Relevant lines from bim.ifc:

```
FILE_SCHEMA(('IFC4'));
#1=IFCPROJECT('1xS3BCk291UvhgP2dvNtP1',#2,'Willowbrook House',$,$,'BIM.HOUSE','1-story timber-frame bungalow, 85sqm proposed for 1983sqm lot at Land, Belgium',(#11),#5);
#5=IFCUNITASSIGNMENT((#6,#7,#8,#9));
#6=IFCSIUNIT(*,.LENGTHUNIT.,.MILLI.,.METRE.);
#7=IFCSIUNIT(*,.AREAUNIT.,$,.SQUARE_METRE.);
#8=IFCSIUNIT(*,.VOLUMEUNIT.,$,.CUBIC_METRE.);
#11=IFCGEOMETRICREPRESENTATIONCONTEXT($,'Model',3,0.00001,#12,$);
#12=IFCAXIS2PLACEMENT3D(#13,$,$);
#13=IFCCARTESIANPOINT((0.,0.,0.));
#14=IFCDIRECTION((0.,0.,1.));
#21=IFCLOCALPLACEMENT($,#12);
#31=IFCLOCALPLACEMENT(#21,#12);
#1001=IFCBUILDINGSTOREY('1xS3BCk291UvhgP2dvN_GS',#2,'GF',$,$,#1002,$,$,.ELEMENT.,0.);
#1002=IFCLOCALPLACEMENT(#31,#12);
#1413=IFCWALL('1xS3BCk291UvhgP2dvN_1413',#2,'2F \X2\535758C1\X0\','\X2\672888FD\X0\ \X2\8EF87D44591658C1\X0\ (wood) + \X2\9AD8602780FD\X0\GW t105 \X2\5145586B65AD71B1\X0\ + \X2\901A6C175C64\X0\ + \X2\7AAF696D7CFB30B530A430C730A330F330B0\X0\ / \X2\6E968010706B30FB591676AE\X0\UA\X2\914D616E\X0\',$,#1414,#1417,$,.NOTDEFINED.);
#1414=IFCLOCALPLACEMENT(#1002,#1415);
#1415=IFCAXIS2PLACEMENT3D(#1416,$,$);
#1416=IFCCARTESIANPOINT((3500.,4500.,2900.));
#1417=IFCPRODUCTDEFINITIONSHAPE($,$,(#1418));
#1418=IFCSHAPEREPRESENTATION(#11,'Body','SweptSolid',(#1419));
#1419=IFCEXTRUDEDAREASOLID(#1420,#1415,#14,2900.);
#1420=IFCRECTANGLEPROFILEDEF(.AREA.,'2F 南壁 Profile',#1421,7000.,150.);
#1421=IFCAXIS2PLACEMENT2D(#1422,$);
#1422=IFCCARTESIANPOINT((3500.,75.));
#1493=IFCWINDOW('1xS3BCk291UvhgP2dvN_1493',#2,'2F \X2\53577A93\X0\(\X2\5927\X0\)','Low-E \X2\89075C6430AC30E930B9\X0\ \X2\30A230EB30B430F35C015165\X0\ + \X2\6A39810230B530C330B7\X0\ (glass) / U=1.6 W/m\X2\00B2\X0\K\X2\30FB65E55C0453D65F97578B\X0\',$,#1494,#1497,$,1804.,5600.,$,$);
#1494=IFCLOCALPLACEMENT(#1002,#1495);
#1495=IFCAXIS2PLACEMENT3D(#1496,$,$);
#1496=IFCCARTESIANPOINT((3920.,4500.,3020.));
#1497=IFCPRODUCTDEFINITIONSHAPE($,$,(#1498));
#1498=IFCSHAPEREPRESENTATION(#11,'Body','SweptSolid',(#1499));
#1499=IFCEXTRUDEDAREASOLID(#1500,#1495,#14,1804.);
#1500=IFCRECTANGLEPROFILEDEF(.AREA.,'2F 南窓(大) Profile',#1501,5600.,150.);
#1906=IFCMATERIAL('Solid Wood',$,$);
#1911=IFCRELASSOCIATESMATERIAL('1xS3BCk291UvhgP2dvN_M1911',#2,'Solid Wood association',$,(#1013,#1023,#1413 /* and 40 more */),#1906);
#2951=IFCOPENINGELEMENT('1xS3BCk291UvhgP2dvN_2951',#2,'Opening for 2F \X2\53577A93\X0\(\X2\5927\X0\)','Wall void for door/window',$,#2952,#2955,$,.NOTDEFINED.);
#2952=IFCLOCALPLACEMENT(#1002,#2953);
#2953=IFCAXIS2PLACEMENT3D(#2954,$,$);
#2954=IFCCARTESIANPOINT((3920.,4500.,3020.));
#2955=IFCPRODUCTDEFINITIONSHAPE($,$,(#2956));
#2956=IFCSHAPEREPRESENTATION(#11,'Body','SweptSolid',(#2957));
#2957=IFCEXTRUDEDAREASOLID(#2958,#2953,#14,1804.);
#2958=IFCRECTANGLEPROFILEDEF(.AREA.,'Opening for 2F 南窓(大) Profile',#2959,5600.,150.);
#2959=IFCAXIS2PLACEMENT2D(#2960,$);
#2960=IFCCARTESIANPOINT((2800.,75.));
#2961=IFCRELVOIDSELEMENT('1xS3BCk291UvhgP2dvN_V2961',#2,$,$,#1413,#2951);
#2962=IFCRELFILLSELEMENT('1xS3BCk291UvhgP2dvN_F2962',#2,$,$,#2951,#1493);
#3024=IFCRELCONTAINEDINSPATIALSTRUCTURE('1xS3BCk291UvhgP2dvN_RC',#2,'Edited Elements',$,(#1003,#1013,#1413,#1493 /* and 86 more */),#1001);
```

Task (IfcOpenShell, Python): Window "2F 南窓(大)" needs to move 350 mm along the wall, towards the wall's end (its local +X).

```python
import ifcopenshell
import ifcopenshell.api.geometry
import ifcopenshell.util.placement
import ifcopenshell.util.unit

model = ifcopenshell.open("bim.ifc")
unit_scale = ifcopenshell.util.unit.calculate_unit_scale(model)

window = model.by_id(1493)
opening = window.FillsVoids[0].RelatingOpeningElement
wall = opening.VoidsElements[0].RelatingBuildingElement

wall_matrix = ifcopenshell.util.placement.get_local_placement(wall.ObjectPlacement)
shift = wall_matrix[:3, 0] * 0.35 / unit_scale
before = ifcopenshell.util.placement.get_local_placement(window.ObjectPlacement)[:3, 3].copy()

# The window is not placed relative to its opening, so move both.
for product in (opening, window):
    matrix = ifcopenshell.util.placement.get_local_placement(product.ObjectPlacement)
    matrix[:3, 3] += shift
    ifcopenshell.api.geometry.edit_object_placement(model, product=product, matrix=matrix, is_si=False)

after = ifcopenshell.util.placement.get_local_placement(window.ObjectPlacement)[:3, 3]
print("window moved by", (after - before).round(3) + 0.0)

model.write("bim_edited.ifc")
```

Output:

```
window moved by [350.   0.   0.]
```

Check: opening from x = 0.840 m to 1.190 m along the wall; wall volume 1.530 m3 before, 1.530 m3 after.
